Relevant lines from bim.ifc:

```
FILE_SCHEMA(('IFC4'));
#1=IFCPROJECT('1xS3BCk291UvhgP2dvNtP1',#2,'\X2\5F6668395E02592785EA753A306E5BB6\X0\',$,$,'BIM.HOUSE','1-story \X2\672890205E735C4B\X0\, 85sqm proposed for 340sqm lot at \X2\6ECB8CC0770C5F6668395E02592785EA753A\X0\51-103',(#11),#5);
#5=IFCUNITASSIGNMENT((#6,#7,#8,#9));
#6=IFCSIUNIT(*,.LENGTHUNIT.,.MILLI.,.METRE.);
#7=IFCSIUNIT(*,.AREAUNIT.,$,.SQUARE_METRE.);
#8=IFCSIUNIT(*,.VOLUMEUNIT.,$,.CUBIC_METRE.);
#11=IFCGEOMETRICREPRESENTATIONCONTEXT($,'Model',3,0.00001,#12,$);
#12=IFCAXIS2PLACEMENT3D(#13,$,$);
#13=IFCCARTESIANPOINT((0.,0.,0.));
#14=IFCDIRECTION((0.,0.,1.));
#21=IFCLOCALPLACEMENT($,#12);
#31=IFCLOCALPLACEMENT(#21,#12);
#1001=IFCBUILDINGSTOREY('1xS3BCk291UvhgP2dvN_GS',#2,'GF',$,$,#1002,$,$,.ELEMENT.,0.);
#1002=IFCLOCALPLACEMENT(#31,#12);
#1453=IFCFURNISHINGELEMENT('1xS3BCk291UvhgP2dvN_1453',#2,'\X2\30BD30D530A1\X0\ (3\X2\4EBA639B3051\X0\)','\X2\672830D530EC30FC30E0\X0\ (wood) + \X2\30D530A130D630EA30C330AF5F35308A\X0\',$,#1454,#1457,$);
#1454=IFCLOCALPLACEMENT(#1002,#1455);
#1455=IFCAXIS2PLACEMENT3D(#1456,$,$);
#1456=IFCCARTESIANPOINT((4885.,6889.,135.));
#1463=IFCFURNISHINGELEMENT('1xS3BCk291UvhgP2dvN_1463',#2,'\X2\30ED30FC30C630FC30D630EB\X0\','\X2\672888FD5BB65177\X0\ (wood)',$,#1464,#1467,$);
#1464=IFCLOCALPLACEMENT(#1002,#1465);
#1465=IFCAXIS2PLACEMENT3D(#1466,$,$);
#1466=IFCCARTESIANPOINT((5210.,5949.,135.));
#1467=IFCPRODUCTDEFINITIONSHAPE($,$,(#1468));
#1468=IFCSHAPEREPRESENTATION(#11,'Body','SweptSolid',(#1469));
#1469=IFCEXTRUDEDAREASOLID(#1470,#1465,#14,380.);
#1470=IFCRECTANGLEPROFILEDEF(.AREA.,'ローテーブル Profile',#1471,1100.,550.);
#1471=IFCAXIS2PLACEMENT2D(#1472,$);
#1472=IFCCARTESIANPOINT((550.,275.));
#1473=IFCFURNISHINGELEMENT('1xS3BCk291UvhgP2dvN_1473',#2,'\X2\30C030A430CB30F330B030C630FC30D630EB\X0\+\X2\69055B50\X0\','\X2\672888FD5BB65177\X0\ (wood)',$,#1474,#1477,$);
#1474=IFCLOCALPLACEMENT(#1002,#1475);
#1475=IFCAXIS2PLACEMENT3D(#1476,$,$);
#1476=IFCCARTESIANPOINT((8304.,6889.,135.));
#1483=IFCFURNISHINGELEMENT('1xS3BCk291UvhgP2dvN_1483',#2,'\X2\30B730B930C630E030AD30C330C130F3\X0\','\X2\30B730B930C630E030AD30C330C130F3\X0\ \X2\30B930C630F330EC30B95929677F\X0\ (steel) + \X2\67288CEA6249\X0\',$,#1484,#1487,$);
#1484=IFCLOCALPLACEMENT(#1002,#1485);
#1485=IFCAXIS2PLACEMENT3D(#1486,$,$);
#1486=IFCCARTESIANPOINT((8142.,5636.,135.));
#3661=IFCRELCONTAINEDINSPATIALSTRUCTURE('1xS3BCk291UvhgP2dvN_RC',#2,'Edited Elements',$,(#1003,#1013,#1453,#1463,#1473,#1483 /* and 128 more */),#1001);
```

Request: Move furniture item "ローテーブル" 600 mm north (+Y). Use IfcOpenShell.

```python
import ifcopenshell
import ifcopenshell.api.geometry
import ifcopenshell.util.placement
import ifcopenshell.util.unit

model = ifcopenshell.open("bim.ifc")
unit_scale = ifcopenshell.util.unit.calculate_unit_scale(model)

item = model.by_id(1463)
matrix = ifcopenshell.util.placement.get_local_placement(item.ObjectPlacement)
matrix[1, 3] += 0.6 / unit_scale
ifcopenshell.api.geometry.edit_object_placement(model, product=item, matrix=matrix, is_si=False)

print(ifcopenshell.util.placement.get_local_placement(item.ObjectPlacement).round(3) + 0.0)

model.write("bim_updated.ifc")
```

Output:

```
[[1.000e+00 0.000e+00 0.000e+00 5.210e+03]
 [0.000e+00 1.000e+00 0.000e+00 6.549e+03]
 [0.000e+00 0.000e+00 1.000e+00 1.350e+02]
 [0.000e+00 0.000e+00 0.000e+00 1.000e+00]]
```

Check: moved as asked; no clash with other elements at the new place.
